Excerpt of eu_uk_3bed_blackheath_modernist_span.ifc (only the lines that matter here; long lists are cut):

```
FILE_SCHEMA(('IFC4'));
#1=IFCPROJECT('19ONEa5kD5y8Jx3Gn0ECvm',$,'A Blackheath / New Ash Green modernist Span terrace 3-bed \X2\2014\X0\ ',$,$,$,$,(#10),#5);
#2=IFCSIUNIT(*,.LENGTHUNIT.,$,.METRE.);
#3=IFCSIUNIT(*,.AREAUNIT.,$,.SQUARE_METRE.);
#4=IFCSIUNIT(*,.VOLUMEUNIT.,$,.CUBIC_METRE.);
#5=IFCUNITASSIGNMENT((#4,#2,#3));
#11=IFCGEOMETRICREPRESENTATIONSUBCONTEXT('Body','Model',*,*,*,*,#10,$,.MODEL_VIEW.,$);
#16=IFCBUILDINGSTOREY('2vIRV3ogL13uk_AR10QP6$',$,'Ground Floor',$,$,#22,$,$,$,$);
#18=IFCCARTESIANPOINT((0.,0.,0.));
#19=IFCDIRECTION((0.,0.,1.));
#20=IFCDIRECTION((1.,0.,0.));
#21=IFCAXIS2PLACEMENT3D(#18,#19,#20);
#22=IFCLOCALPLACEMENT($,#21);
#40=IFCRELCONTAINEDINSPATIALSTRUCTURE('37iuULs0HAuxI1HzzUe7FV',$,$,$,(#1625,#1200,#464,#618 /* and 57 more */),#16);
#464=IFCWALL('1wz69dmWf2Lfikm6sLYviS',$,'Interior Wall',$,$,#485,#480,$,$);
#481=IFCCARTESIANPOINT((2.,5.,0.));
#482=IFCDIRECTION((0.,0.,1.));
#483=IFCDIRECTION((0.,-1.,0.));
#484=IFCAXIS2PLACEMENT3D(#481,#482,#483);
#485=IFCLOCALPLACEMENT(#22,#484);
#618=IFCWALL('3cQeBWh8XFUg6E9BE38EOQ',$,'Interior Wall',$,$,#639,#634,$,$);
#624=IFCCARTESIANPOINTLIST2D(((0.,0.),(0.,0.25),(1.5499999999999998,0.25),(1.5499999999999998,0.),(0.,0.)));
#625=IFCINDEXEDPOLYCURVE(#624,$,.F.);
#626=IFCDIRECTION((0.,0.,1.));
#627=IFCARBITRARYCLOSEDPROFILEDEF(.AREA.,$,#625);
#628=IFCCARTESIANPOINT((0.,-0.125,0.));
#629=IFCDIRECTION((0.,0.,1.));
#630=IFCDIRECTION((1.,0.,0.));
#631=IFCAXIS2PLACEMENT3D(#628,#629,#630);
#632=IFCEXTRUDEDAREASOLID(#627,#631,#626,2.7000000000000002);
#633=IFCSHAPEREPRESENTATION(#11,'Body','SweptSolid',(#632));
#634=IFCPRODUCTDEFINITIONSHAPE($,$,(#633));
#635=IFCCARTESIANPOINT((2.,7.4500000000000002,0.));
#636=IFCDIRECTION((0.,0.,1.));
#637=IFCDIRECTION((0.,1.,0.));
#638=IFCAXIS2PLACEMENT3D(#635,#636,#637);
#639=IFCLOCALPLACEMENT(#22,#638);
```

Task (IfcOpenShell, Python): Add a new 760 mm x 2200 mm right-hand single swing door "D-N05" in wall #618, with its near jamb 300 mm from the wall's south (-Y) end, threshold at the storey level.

```python
import numpy as np
import ifcopenshell
import ifcopenshell.api.feature
import ifcopenshell.api.geometry
import ifcopenshell.api.root
import ifcopenshell.api.spatial
import ifcopenshell.geom
import ifcopenshell.util.element
import ifcopenshell.util.placement
import ifcopenshell.util.representation
import ifcopenshell.util.shape
import ifcopenshell.util.unit

model = ifcopenshell.open("eu_uk_3bed_blackheath_modernist_span.ifc")
unit_scale = ifcopenshell.util.unit.calculate_unit_scale(model)
settings = ifcopenshell.geom.settings()


def volume(element):
    """Net volume in cubic metres, openings subtracted."""
    shape = ifcopenshell.geom.create_shape(settings, element)
    return ifcopenshell.util.shape.get_volume(shape.geometry)


wall = model.by_guid("3cQeBWh8XFUg6E9BE38EOQ")
storey = ifcopenshell.util.element.get_container(wall, ifc_class="IfcBuildingStorey")
context = ifcopenshell.util.representation.get_context(model, "Model", "Body", "MODEL_VIEW")
before = volume(wall)

width, height, from_end, sill = 0.76, 2.2, 0.3, 0.0  # metres

# The wall runs along its own X axis, and the end named is its -X end.
wall_shape = ifcopenshell.geom.create_shape(settings, wall)
x, y, z = ifcopenshell.util.shape.get_vertices(wall_shape.geometry).T
start = x.min() + from_end
face, thickness = float(y.min()), float(y.max() - y.min())
wall_matrix = ifcopenshell.util.placement.get_local_placement(wall.ObjectPlacement)
level = ifcopenshell.util.placement.get_local_placement(storey.ObjectPlacement)[2, 3]


def in_wall(x, y):
    """Placement at x, y metres in the wall's axes, at sill height."""
    matrix = wall_matrix.copy()
    matrix[:, 3] = wall_matrix @ np.array([x / unit_scale, y / unit_scale, 0.0, 1.0])
    matrix[2, 3] = level + sill / unit_scale
    return matrix


# Opening: a box that overshoots both wall faces by 50 mm.
opening = ifcopenshell.api.root.create_entity(model, ifc_class="IfcOpeningElement", predefined_type="OPENING")
box = ifcopenshell.api.geometry.add_wall_representation(
    model, context=context, length=width, height=height, thickness=thickness + 0.1
)
ifcopenshell.api.geometry.assign_representation(model, product=opening, representation=box)
ifcopenshell.api.geometry.edit_object_placement(model, product=opening, matrix=in_wall(start, face - 0.05), is_si=False)
ifcopenshell.api.feature.add_feature(model, feature=opening, element=wall)

door = ifcopenshell.api.root.create_entity(model, ifc_class="IfcDoor", name="D-N05", predefined_type="DOOR")
door.OverallWidth, door.OverallHeight = width / unit_scale, height / unit_scale
door.OperationType = "SINGLE_SWING_RIGHT"
body = ifcopenshell.api.geometry.add_door_representation(
    model,
    context=context,
    overall_width=door.OverallWidth,
    overall_height=door.OverallHeight,
    operation_type="SINGLE_SWING_RIGHT",
    lining_properties={"LiningDepth": thickness / unit_scale, "ThresholdDepth": thickness / unit_scale},
)
ifcopenshell.api.geometry.assign_representation(model, product=door, representation=body)
ifcopenshell.api.spatial.assign_container(model, products=[door], relating_structure=storey)
ifcopenshell.api.feature.add_filling(model, opening=opening, element=door)

# The lining spans the wall, so the door starts at the wall face.
ifcopenshell.api.geometry.edit_object_placement(model, product=door, matrix=in_wall(start, face), is_si=False)

after = volume(wall)

print(f"wall volume {before:.3f} -> {after:.3f} m3")

model.write("eu_uk_3bed_blackheath_modernist_span_edited.ifc")
```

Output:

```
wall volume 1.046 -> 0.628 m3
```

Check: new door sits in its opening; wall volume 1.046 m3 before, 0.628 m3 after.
